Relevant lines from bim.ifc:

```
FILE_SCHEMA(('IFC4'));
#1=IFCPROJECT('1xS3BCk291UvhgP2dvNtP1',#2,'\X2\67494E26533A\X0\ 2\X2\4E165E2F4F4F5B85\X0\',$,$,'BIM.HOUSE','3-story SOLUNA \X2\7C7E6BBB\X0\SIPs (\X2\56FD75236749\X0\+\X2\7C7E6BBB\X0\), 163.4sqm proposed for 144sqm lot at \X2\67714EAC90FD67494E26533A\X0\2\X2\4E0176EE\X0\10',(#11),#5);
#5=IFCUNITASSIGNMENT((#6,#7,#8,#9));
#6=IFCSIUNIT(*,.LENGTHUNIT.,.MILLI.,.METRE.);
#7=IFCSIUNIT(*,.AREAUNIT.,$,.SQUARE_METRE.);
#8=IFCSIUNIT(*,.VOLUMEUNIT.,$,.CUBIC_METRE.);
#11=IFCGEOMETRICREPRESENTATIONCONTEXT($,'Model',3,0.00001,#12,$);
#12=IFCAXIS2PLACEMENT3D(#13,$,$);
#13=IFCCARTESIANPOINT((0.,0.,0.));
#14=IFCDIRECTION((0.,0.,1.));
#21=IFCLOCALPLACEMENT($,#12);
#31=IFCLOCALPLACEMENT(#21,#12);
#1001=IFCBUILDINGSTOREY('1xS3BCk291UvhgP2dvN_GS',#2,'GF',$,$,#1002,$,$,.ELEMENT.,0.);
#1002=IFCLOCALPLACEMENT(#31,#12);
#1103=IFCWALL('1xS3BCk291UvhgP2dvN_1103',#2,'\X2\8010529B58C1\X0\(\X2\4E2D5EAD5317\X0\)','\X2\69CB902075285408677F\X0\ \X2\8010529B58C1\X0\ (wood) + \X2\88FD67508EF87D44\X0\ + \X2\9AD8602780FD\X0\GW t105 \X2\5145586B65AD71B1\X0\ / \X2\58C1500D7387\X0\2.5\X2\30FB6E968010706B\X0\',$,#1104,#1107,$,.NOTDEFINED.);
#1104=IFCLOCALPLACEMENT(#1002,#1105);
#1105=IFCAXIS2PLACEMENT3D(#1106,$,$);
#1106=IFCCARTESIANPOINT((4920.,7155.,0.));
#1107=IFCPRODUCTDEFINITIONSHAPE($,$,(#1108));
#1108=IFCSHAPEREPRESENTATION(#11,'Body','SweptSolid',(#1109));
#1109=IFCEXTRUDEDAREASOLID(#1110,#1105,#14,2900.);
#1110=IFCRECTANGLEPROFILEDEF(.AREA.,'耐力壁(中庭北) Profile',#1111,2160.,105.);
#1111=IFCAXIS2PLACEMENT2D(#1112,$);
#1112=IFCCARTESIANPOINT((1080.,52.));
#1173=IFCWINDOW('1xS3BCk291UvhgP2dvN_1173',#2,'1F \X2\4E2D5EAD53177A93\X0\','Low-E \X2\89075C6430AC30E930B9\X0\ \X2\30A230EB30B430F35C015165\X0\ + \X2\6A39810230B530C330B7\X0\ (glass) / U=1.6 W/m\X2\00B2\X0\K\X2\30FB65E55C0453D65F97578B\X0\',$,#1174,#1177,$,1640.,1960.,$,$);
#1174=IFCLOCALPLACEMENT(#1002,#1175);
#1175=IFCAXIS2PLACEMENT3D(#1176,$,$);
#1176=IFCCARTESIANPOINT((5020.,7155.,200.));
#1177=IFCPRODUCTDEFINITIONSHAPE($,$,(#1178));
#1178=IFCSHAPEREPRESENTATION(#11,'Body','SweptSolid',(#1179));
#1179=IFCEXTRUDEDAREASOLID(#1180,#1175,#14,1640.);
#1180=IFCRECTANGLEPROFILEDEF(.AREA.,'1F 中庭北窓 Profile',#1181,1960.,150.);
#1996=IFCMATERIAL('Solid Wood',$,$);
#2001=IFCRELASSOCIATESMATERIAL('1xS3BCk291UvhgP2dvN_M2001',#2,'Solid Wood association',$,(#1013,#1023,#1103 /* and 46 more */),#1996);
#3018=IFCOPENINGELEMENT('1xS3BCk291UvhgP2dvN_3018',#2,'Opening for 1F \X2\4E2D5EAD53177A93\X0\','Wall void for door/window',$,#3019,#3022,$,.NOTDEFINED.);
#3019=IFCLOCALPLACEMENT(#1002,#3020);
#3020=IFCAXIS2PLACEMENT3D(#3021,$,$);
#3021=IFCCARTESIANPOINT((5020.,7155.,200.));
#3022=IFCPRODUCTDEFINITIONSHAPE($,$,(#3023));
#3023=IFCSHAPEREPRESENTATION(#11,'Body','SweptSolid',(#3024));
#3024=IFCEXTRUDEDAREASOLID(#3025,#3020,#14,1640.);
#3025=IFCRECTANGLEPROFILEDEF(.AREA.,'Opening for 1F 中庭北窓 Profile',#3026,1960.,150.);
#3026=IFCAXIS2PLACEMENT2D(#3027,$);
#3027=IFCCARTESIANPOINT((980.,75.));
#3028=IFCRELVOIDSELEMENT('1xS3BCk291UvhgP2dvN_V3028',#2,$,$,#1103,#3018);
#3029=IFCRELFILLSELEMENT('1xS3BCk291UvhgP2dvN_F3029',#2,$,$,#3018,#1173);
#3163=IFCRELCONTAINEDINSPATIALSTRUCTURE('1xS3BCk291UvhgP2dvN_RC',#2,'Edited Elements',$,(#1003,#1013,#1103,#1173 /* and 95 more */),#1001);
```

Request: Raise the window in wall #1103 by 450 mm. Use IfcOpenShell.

```python
import numpy as np
import ifcopenshell
import ifcopenshell.api.geometry
import ifcopenshell.util.placement
import ifcopenshell.util.unit

model = ifcopenshell.open("bim.ifc")
unit_scale = ifcopenshell.util.unit.calculate_unit_scale(model)

window = model.by_guid("1xS3BCk291UvhgP2dvN_1173")
opening = window.FillsVoids[0].RelatingOpeningElement
dz = 0.45 / unit_scale

shift = np.array([0.0, 0.0, dz])
# The window is not placed relative to its opening, so move both.
for product in (opening, window):
    matrix = ifcopenshell.util.placement.get_local_placement(product.ObjectPlacement)
    matrix[:3, 3] += shift
    ifcopenshell.api.geometry.edit_object_placement(model, product=product, matrix=matrix, is_si=False)

print(f"moved by {dz * unit_scale:+.3f} m")

model.write("bim_v2.ifc")
```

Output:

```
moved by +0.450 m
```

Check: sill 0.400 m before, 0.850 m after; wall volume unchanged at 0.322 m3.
